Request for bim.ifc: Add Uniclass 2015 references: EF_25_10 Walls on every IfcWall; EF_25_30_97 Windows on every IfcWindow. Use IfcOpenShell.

First a look at what the model holds.

```python
import ifcopenshell

model = ifcopenshell.open("bim.ifc")
print(model.schema)
print("classifications:", [c.Name for c in model.by_type("IfcClassification")])
for ifc_class in ("IfcDoor", "IfcRoof", "IfcStair", "IfcWall", "IfcWindow"):
    print(ifc_class, len(model.by_type(ifc_class)))
```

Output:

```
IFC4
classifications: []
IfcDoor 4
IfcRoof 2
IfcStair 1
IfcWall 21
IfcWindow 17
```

```python
import ifcopenshell
import ifcopenshell.api.classification

model = ifcopenshell.open("bim.ifc")

system = ifcopenshell.api.classification.add_classification(model, classification="Uniclass 2015")

codes = {
    "IfcWall": ("EF_25_10", "Walls"),
    "IfcWindow": ("EF_25_30_97", "Windows"),
}
for ifc_class, (code, name) in codes.items():
    products = model.by_type(ifc_class)
    ifcopenshell.api.classification.add_reference(
        model, products=products, classification=system, identification=code, name=name
    )
    print(code, len(products))

model.write("bim_updated.ifc")
```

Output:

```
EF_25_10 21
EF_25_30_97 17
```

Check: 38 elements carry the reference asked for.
